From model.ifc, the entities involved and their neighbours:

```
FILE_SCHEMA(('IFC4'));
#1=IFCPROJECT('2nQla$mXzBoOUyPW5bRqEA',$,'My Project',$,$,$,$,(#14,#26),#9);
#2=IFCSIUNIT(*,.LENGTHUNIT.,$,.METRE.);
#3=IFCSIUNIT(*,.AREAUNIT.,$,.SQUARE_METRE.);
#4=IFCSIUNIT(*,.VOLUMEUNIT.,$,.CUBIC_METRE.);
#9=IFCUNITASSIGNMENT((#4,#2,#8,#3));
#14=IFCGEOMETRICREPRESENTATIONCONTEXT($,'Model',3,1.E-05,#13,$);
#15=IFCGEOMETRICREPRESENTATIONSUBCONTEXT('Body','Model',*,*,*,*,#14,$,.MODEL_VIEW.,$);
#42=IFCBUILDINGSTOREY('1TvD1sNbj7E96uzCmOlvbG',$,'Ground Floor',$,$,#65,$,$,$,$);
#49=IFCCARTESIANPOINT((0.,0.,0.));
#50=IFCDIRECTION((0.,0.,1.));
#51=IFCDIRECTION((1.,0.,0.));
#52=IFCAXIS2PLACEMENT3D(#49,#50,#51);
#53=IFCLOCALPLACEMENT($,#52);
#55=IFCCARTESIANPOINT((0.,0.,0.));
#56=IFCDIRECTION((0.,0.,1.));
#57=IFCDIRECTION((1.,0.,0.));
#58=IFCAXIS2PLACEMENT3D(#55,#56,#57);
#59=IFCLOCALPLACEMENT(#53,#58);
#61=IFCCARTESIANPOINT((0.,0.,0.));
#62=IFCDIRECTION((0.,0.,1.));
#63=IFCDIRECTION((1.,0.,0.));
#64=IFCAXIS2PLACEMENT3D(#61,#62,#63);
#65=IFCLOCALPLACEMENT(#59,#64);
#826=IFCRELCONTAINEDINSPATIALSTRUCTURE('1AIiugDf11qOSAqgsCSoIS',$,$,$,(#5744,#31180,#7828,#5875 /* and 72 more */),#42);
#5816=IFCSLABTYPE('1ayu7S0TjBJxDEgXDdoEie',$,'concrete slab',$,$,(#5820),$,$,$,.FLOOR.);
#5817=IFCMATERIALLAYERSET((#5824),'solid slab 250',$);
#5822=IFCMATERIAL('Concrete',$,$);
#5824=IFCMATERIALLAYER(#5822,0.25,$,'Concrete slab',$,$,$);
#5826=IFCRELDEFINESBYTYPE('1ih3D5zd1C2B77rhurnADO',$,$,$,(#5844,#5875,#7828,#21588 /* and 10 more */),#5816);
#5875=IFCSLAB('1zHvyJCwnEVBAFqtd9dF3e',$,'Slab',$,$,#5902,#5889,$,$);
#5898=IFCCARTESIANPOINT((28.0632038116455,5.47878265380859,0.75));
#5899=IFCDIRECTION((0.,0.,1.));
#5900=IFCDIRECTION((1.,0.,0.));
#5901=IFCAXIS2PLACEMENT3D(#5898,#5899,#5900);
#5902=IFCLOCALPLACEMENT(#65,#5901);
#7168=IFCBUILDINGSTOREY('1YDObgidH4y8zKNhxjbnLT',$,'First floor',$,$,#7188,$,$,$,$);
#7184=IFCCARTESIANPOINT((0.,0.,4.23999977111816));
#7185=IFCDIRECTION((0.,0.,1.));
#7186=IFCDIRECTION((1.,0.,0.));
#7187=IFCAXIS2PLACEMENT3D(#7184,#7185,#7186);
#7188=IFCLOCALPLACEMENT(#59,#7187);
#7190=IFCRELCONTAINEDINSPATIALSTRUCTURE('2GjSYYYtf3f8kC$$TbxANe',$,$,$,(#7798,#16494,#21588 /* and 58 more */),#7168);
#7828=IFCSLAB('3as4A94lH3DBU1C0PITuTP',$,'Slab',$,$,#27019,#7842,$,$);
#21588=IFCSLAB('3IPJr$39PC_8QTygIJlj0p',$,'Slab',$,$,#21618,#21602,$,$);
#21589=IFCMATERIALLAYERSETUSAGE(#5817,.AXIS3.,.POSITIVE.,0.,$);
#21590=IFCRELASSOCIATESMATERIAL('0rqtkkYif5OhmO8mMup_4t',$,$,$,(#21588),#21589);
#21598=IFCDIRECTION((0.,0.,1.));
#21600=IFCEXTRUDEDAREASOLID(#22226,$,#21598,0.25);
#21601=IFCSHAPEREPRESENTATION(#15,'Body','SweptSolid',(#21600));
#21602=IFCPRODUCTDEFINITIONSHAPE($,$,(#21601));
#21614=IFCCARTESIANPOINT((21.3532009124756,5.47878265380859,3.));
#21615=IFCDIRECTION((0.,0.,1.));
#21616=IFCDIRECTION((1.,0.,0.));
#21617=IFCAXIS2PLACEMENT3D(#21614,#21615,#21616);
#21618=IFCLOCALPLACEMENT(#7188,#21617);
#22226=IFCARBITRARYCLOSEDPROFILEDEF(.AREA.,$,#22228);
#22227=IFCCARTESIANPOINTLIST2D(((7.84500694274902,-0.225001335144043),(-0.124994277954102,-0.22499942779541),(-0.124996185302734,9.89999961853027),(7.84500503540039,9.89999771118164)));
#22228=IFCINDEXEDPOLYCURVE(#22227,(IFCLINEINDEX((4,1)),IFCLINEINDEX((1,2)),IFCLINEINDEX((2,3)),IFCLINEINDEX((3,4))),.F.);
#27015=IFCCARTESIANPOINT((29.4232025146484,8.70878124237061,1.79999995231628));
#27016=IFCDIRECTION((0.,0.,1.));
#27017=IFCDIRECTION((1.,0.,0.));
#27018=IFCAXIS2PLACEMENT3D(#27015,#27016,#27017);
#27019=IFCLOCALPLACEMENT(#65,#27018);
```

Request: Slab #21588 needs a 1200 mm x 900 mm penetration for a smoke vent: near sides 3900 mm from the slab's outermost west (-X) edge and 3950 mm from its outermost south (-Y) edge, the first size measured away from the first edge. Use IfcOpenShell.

```python
import numpy as np
import ifcopenshell
import ifcopenshell.api.feature
import ifcopenshell.api.geometry
import ifcopenshell.api.root
import ifcopenshell.geom
import ifcopenshell.util.placement
import ifcopenshell.util.representation
import ifcopenshell.util.shape
import ifcopenshell.util.unit

model = ifcopenshell.open("model.ifc")
unit_scale = ifcopenshell.util.unit.calculate_unit_scale(model)
settings = ifcopenshell.geom.settings()


def volume(element):
    """Net volume in cubic metres, openings subtracted."""
    shape = ifcopenshell.geom.create_shape(settings, element)
    return ifcopenshell.util.shape.get_volume(shape.geometry)


slab = model.by_guid("3IPJr$39PC_8QTygIJlj0p")
before = volume(slab)

# Extent in the slab's own axes, in metres. The edges named are its -X and -Y sides.
slab_shape = ifcopenshell.geom.create_shape(settings, slab)
vertices = ifcopenshell.util.shape.get_vertices(slab_shape.geometry)
x_min, y_min, bottom = vertices.min(axis=0)
top = vertices[:, 2].max()

opening = ifcopenshell.api.root.create_entity(model, ifc_class="IfcOpeningElement", name="Smoke vent opening", predefined_type="OPENING")
context = ifcopenshell.util.representation.get_context(model, "Model", "Body", "MODEL_VIEW")
width, depth = 1.2, 0.9
outline = [(0.0, 0.0), (width, 0.0), (width, depth), (0.0, depth), (0.0, 0.0)]
# Overshoot both faces by 50 mm so the cut is clean.
shape = ifcopenshell.api.geometry.add_slab_representation(
    model, context=context, depth=top - bottom + 0.1, polyline=outline
)
ifcopenshell.api.geometry.assign_representation(model, product=opening, representation=shape)

matrix = ifcopenshell.util.placement.get_local_placement(slab.ObjectPlacement)
matrix[:, 3] = matrix @ np.append(np.array([x_min + 3.9, y_min + 3.95, bottom - 0.05]) / unit_scale, 1.0)
ifcopenshell.api.geometry.edit_object_placement(model, product=opening, matrix=matrix, is_si=False)
ifcopenshell.api.feature.add_feature(model, feature=opening, element=slab)

after = volume(slab)

print(f"slab volume {before:.3f} -> {after:.3f} m3")

model.write("model_edited.ifc")
```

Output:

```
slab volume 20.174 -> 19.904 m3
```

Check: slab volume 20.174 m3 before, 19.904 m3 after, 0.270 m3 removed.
